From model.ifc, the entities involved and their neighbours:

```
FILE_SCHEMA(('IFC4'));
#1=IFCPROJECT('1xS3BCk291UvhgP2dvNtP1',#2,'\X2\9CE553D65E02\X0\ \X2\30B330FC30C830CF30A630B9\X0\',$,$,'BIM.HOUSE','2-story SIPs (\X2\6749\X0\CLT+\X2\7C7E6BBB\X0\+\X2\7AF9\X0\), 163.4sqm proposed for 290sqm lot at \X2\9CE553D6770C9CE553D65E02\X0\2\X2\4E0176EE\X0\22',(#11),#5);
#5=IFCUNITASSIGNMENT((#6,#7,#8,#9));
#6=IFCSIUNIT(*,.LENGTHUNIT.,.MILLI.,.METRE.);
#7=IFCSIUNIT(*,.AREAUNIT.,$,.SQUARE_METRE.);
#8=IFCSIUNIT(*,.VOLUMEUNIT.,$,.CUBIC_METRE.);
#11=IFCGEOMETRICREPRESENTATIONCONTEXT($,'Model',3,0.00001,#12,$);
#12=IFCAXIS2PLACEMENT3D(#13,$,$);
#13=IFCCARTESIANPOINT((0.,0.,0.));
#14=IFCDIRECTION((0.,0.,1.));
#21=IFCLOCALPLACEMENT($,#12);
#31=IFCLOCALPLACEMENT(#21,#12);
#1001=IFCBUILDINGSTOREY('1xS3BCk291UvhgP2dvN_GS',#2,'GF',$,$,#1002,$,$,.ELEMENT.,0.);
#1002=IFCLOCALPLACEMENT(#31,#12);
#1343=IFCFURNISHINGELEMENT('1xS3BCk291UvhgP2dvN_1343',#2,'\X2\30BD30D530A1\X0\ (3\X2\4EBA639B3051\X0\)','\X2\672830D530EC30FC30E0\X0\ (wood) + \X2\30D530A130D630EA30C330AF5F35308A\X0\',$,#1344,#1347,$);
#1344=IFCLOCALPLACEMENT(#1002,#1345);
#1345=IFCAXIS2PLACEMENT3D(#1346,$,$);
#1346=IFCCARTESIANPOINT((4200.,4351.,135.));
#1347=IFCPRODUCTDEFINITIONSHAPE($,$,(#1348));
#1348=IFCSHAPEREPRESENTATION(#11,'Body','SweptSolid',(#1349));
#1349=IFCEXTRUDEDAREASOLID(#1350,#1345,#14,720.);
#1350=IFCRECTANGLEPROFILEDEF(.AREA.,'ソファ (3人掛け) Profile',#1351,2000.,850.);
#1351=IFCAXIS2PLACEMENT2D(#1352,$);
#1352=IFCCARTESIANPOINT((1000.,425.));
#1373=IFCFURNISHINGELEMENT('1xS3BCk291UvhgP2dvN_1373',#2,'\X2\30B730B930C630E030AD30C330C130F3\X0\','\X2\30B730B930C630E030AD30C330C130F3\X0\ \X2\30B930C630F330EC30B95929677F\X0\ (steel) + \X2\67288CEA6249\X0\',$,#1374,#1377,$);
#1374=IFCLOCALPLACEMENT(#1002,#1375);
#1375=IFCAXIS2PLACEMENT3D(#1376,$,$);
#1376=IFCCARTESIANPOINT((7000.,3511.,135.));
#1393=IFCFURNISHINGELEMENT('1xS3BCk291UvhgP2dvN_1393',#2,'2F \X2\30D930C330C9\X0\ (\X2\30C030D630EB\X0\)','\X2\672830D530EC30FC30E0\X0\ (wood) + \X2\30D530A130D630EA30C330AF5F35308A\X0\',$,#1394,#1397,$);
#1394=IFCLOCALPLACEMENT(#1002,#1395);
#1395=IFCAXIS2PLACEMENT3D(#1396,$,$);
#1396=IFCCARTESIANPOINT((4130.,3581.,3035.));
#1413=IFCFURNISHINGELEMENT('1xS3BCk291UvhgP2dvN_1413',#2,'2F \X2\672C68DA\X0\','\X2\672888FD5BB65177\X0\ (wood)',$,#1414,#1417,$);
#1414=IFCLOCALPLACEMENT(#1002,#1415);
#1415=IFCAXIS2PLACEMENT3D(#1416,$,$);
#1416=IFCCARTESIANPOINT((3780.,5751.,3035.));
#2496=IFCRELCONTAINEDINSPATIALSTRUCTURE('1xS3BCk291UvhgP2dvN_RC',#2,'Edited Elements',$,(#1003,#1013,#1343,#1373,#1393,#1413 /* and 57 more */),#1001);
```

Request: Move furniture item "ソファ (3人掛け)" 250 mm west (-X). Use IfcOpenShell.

```python
import ifcopenshell
import ifcopenshell.api.geometry
import ifcopenshell.util.placement

model = ifcopenshell.open("model.ifc")

item = model.by_guid("1xS3BCk291UvhgP2dvN_1343")
matrix = ifcopenshell.util.placement.get_local_placement(item.ObjectPlacement)
matrix[0, 3] -= 250.0
ifcopenshell.api.geometry.edit_object_placement(model, product=item, matrix=matrix, is_si=False)

print(ifcopenshell.util.placement.get_local_placement(item.ObjectPlacement).round(3) + 0.0)

model.write("model_rev.ifc")
```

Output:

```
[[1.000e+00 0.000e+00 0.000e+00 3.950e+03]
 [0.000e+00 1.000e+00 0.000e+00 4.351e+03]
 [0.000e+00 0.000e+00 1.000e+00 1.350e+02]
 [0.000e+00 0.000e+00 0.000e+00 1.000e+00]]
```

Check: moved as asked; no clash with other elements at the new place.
